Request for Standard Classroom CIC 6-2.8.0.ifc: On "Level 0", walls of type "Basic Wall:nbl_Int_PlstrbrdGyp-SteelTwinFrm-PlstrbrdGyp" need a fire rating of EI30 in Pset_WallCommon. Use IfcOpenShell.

First a look at what the model holds.

```python
import ifcopenshell
import ifcopenshell.util.element

model = ifcopenshell.open("Standard Classroom CIC 6-2.8.0.ifc")
print(model.schema)
storey = next(s for s in model.by_type("IfcBuildingStorey") if s.Name == "Level 0")
walls = [e for e in ifcopenshell.util.element.get_decomposition(storey) if e.is_a("IfcWall")]
seen = {}
for e in walls:
    element_type = ifcopenshell.util.element.get_type(e)
    key = (element_type.Name if element_type != e and element_type else None, ifcopenshell.util.element.get_pset(e, "Pset_WallCommon", "FireRating"))
    seen[key] = seen.get(key, 0) + 1
for (name, value), count in sorted(seen.items(), key=str):
    print(count, "x", name, "|", value)
```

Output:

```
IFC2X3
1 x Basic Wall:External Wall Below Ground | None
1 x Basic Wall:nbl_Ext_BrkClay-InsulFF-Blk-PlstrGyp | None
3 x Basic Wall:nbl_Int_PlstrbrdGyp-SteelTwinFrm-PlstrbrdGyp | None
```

```python
import ifcopenshell
import ifcopenshell.api.pset
import ifcopenshell.util.element

model = ifcopenshell.open("Standard Classroom CIC 6-2.8.0.ifc")

storey = next(s for s in model.by_type("IfcBuildingStorey") if s.Name == "Level 0")
walls = [e for e in ifcopenshell.util.element.get_decomposition(storey) if e.is_a("IfcWall")]

count = 0
for e in walls:
    element_type = ifcopenshell.util.element.get_type(e)
    if element_type in (None, e) or element_type.Name != "Basic Wall:nbl_Int_PlstrbrdGyp-SteelTwinFrm-PlstrbrdGyp":
        continue
    # add_pset returns the element's existing set when there is one.
    pset = ifcopenshell.api.pset.add_pset(model, product=e, name="Pset_WallCommon")
    ifcopenshell.api.pset.edit_pset(model, pset=pset, properties={"FireRating": "EI30"})
    count += 1

print(count, "walls updated")

model.write("Standard Classroom CIC 6-2.8.0-out.ifc")
```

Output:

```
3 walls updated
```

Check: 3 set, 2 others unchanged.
